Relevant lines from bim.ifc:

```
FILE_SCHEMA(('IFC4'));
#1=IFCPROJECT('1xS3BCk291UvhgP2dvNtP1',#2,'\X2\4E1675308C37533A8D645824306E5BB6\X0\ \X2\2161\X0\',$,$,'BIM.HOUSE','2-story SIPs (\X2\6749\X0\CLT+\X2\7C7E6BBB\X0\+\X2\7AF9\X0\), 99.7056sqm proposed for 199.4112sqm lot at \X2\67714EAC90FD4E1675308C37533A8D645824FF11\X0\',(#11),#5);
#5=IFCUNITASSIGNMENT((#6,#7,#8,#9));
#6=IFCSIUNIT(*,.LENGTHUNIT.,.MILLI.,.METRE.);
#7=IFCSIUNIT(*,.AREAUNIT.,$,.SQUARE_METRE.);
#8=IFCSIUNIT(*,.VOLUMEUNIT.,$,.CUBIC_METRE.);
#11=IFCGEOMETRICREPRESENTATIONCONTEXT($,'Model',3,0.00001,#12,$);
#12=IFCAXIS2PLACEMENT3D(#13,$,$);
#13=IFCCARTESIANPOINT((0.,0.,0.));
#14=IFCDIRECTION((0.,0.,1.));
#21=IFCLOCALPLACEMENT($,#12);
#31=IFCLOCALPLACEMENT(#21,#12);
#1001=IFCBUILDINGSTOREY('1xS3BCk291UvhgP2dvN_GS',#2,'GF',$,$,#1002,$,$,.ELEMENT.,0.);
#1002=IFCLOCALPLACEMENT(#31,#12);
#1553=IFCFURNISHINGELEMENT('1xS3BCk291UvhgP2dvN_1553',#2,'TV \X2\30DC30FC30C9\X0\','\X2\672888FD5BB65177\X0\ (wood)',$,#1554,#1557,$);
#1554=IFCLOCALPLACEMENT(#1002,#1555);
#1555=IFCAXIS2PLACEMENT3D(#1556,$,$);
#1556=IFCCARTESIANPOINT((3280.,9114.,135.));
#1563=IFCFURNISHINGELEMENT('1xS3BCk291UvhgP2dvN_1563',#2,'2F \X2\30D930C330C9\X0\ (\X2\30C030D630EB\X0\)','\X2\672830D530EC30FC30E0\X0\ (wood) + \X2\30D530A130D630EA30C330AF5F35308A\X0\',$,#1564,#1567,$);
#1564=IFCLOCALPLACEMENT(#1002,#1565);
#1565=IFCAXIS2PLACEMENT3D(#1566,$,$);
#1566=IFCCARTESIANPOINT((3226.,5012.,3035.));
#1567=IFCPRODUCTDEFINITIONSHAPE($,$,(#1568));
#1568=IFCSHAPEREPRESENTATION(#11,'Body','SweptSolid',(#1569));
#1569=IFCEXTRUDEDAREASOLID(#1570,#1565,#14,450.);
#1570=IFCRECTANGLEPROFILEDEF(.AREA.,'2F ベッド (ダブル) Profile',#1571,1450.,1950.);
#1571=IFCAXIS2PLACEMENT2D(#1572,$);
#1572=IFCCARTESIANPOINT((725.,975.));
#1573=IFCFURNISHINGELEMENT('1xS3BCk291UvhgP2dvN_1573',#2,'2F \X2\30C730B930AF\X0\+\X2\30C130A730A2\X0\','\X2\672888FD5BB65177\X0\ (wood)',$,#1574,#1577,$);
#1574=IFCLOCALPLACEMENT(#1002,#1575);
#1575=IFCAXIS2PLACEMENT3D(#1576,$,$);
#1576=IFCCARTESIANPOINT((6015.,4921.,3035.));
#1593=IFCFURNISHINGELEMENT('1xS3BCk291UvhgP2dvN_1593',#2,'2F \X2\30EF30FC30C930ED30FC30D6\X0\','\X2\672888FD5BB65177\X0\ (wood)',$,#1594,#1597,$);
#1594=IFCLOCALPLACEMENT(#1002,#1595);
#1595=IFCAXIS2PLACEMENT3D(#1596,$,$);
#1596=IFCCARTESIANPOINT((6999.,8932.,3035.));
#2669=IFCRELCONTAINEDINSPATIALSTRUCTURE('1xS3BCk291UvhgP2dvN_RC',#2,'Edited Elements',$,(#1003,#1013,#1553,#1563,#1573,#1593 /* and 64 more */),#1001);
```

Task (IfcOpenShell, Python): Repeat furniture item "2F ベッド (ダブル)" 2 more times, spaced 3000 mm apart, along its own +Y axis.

```python
import ifcopenshell
import ifcopenshell.api.geometry
import ifcopenshell.api.root
import ifcopenshell.util.element
import ifcopenshell.util.placement
import ifcopenshell.util.unit

model = ifcopenshell.open("bim.ifc")
unit_scale = ifcopenshell.util.unit.calculate_unit_scale(model)


def reuse_history(source, copy):
    """copy_class also copies each property set's owner history, people and application; keep the originals."""
    for rel in copy.IsDefinedBy:
        if rel.is_a("IfcRelDefinesByProperties") and (history := rel.RelatingPropertyDefinition.OwnerHistory):
            rel.RelatingPropertyDefinition.OwnerHistory = source.OwnerHistory
            ifcopenshell.util.element.remove_deep2(model, history)


source = model.by_id(1563)
base = ifcopenshell.util.placement.get_local_placement(source.ObjectPlacement)
step = base[:3, 1] * 3 / unit_scale

for i in range(1, 3):
    copy = ifcopenshell.api.root.copy_class(model, product=source)
    copy.Representation = ifcopenshell.util.element.copy_deep(
        model, source.Representation, exclude=["IfcGeometricRepresentationContext", "IfcRepresentationMap"]
    )
    reuse_history(source, copy)
    matrix = base.copy()
    matrix[:3, 3] += i * step
    print("added at", matrix[:3, 3].round(3) + 0.0)
    ifcopenshell.api.geometry.edit_object_placement(model, product=copy, matrix=matrix, is_si=False)

model.write("bim_v2.ifc")
```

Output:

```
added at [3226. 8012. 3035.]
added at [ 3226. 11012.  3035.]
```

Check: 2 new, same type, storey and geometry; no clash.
